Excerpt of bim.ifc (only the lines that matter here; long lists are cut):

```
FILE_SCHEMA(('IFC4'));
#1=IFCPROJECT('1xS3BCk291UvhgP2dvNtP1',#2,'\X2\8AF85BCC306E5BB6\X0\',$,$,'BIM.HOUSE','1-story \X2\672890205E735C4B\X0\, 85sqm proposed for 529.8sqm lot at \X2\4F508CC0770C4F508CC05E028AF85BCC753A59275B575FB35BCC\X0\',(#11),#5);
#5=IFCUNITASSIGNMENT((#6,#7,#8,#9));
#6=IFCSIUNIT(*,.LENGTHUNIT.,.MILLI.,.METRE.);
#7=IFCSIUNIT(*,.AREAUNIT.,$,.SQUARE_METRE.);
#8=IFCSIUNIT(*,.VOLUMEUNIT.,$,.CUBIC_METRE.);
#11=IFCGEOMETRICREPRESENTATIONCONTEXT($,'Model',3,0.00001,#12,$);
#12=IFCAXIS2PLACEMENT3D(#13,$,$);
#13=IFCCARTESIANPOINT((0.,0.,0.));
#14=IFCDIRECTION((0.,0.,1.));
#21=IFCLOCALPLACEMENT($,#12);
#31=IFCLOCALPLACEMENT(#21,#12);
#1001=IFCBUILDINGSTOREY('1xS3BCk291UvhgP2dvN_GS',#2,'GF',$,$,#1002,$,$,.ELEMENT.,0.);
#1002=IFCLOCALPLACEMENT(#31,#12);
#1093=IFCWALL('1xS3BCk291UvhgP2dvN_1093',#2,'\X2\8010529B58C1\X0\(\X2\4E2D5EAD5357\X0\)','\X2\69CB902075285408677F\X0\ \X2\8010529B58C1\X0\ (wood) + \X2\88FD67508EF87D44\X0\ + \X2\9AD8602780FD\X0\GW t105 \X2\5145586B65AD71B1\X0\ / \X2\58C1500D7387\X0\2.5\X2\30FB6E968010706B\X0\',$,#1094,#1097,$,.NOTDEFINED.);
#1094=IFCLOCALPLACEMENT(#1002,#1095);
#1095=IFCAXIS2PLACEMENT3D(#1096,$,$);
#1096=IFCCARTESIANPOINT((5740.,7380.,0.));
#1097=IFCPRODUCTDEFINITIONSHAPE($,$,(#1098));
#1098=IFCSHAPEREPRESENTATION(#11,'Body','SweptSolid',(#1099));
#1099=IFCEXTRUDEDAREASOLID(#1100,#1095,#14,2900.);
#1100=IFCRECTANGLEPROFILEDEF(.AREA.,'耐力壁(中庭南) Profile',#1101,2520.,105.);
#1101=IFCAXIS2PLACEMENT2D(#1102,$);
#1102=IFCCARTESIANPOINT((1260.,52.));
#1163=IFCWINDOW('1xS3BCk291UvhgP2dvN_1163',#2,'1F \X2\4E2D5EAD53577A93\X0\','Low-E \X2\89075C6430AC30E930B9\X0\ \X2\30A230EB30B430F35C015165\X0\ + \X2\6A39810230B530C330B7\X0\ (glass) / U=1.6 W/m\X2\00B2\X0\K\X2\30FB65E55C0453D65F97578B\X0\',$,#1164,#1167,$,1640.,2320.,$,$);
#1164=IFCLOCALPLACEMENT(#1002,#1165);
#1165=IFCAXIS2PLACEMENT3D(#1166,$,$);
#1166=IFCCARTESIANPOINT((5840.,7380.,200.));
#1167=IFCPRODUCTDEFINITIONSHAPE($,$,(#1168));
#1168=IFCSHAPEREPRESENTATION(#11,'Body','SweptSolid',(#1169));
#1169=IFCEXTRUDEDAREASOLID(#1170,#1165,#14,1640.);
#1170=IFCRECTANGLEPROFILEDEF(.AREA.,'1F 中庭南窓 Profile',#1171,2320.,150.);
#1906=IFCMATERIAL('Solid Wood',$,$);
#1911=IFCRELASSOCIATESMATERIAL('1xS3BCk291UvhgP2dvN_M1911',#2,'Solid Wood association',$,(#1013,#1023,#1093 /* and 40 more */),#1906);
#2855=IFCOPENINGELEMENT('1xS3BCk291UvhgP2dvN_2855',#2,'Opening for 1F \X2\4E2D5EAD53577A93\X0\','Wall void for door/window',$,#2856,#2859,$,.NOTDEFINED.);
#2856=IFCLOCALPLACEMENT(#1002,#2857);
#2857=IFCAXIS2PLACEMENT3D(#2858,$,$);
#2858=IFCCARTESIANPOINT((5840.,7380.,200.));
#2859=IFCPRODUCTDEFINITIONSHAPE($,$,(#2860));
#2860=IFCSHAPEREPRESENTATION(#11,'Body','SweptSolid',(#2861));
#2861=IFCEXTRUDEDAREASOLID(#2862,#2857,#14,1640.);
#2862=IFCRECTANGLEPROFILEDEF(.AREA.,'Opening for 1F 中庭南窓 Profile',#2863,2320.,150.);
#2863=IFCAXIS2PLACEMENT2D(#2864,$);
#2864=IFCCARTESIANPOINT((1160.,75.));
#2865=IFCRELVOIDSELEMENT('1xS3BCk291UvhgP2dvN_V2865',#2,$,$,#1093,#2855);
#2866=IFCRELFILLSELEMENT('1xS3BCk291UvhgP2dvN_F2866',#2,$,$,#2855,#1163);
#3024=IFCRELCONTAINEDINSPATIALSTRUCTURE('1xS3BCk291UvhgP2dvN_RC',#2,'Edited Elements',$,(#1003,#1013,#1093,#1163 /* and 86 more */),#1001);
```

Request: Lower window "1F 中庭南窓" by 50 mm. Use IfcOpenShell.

```python
import numpy as np
import ifcopenshell
import ifcopenshell.api.geometry
import ifcopenshell.util.placement
import ifcopenshell.util.unit

model = ifcopenshell.open("bim.ifc")
unit_scale = ifcopenshell.util.unit.calculate_unit_scale(model)

window = model.by_guid("1xS3BCk291UvhgP2dvN_1163")
opening = window.FillsVoids[0].RelatingOpeningElement
dz = -50.0

shift = np.array([0.0, 0.0, dz])
# The window is not placed relative to its opening, so move both.
for product in (opening, window):
    matrix = ifcopenshell.util.placement.get_local_placement(product.ObjectPlacement)
    matrix[:3, 3] += shift
    ifcopenshell.api.geometry.edit_object_placement(model, product=product, matrix=matrix, is_si=False)

print(f"moved by {dz * unit_scale:+.3f} m")

model.write("bim_updated.ifc")
```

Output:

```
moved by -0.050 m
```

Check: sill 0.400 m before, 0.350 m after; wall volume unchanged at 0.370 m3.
